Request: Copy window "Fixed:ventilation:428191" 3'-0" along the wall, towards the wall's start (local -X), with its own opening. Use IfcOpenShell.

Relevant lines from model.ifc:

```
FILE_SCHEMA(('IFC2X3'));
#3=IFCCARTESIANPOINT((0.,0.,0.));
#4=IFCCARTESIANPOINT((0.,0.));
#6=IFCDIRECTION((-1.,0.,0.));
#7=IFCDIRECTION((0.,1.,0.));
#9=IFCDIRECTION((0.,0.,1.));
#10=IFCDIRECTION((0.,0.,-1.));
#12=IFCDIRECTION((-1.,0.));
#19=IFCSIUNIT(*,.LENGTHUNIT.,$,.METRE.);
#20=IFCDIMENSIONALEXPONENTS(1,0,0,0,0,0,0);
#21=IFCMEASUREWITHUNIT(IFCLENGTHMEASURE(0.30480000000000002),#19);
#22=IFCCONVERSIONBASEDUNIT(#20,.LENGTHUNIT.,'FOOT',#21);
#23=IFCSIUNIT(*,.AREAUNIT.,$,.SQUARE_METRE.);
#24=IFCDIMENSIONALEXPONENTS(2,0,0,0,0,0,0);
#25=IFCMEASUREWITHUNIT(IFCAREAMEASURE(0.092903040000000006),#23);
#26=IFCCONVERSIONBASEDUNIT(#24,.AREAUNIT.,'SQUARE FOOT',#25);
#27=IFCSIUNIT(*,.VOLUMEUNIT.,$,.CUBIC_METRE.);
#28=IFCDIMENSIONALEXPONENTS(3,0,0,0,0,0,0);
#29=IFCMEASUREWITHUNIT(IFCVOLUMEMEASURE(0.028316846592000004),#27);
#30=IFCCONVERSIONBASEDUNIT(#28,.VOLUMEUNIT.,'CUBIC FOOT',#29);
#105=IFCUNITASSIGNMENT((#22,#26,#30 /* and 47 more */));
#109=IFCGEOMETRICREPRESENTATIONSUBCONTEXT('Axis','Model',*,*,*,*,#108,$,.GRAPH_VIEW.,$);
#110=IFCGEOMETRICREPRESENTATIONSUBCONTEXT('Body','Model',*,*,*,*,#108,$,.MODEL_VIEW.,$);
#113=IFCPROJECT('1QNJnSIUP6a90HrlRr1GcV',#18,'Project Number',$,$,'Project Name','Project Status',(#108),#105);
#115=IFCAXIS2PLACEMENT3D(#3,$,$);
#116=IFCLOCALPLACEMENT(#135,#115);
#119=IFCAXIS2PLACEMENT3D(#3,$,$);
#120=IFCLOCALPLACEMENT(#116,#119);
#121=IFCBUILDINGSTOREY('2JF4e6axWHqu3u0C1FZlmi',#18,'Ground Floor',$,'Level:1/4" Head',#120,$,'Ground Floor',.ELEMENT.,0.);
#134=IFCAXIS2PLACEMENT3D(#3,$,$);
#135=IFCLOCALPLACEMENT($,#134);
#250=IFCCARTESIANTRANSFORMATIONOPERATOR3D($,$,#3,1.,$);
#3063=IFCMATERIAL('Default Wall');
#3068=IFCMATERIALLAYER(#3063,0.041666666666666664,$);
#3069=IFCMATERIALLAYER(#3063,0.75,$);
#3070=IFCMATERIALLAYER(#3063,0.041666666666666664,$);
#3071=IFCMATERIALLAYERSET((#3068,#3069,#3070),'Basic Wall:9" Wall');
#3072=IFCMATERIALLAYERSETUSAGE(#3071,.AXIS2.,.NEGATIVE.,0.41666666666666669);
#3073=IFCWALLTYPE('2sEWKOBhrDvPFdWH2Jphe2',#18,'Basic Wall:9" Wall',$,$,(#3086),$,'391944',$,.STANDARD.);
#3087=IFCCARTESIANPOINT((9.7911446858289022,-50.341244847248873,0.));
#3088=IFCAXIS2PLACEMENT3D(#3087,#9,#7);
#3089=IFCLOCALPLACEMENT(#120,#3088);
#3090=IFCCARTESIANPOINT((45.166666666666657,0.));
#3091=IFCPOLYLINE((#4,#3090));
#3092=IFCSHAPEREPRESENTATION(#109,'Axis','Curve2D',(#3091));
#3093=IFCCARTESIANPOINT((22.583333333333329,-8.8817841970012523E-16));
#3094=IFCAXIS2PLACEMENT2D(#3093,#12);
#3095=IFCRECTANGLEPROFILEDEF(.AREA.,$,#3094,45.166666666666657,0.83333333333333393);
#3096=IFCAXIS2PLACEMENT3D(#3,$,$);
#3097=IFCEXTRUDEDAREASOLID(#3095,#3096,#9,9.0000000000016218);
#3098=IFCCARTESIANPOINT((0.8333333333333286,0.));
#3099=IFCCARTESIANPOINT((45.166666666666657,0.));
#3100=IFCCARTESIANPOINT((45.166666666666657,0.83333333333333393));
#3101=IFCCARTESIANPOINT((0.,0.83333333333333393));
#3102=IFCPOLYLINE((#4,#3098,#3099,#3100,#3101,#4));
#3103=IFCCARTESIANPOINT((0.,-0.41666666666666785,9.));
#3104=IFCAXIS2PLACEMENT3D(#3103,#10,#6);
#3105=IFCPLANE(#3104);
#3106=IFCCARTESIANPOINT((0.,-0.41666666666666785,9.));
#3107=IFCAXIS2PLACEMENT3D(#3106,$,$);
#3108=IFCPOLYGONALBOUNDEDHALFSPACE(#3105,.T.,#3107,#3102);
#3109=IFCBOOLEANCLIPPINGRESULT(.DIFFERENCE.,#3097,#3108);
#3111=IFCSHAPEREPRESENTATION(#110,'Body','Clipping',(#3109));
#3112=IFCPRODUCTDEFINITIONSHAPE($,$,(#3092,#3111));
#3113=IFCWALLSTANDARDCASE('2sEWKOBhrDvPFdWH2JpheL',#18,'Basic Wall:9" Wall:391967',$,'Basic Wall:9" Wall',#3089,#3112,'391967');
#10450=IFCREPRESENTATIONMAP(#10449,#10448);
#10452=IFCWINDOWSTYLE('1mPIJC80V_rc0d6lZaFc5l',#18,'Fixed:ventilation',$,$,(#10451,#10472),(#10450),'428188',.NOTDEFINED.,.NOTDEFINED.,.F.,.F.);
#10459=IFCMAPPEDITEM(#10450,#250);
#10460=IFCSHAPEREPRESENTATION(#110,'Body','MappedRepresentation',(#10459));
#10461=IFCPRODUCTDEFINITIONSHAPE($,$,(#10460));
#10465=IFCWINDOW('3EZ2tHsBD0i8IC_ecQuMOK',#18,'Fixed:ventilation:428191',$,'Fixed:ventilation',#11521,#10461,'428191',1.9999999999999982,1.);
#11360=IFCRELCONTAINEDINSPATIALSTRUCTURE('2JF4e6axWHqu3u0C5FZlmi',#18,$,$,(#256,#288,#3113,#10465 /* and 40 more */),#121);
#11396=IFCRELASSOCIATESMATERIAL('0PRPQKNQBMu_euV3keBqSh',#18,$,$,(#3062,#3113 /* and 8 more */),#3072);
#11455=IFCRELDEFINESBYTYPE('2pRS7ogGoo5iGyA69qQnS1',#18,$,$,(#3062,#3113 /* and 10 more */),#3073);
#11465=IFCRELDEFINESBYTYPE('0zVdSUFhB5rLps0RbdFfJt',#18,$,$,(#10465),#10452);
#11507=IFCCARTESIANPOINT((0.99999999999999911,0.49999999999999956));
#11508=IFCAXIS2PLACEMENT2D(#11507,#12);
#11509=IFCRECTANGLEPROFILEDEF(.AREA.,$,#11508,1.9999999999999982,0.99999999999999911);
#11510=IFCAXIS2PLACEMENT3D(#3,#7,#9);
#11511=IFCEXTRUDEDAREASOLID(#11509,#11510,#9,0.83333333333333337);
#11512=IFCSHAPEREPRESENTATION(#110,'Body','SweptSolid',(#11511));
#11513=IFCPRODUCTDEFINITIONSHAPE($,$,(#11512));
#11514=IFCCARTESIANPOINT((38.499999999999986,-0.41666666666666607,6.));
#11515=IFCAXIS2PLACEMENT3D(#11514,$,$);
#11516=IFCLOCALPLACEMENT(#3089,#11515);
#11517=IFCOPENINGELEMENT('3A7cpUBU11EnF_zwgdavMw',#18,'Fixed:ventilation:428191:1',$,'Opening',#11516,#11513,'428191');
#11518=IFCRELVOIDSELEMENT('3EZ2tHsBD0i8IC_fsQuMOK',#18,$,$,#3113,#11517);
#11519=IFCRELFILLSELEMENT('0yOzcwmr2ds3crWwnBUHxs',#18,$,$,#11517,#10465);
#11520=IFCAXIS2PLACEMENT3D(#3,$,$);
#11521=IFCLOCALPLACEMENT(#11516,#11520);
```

```python
import ifcopenshell
import ifcopenshell.api.feature
import ifcopenshell.api.geometry
import ifcopenshell.api.root
import ifcopenshell.geom
import ifcopenshell.util.element
import ifcopenshell.util.placement
import ifcopenshell.util.shape
import ifcopenshell.util.unit

model = ifcopenshell.open("model.ifc")
unit_scale = ifcopenshell.util.unit.calculate_unit_scale(model)
settings = ifcopenshell.geom.settings()


def volume(element):
    """Net volume in cubic metres, openings subtracted."""
    shape = ifcopenshell.geom.create_shape(settings, element)
    return ifcopenshell.util.shape.get_volume(shape.geometry)


def reuse_history(source, copy):
    """copy_class also copies each property set's owner history, people and application; keep the originals."""
    for rel in copy.IsDefinedBy:
        if rel.is_a("IfcRelDefinesByProperties") and (history := rel.RelatingPropertyDefinition.OwnerHistory):
            rel.RelatingPropertyDefinition.OwnerHistory = source.OwnerHistory
            ifcopenshell.util.element.remove_deep2(model, history)


window = model.by_guid("3EZ2tHsBD0i8IC_ecQuMOK")
opening = window.FillsVoids[0].RelatingOpeningElement
wall = opening.VoidsElements[0].RelatingBuildingElement
before = volume(wall)
shift = ifcopenshell.util.placement.get_local_placement(wall.ObjectPlacement)[:3, 0] * -36 * 0.0254 / unit_scale

# copy_class copies the void relationship, type, container and properties, but no geometry.
new_opening = ifcopenshell.api.root.copy_class(model, product=opening)
new_opening.Representation = ifcopenshell.util.element.copy_deep(
    model, opening.Representation, exclude=["IfcGeometricRepresentationContext", "IfcRepresentationMap"]
)
new_opening.Name = "Fixed:ventilation"
new_opening.Tag = None
new_window = ifcopenshell.api.root.copy_class(model, product=window)
new_window.Representation = ifcopenshell.util.element.copy_deep(
    model, window.Representation, exclude=["IfcGeometricRepresentationContext", "IfcRepresentationMap"]
)
new_window.Name = "Fixed:ventilation"
new_window.Tag = None
reuse_history(window, new_window)
fills = ifcopenshell.api.feature.add_filling(model, opening=new_opening, element=new_window)
fills.OwnerHistory = new_window.OwnerHistory  # required in IFC2X3

for old, new in ((opening, new_opening), (window, new_window)):
    matrix = ifcopenshell.util.placement.get_local_placement(old.ObjectPlacement)
    matrix[:3, 3] += shift
    ifcopenshell.api.geometry.edit_object_placement(model, product=new, matrix=matrix, is_si=False)

after = volume(wall)

print(f"wall volume {before:.3f} -> {after:.3f} m3")

model.write("model-out.ifc")
```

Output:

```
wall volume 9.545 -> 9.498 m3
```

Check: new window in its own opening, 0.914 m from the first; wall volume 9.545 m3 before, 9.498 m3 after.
